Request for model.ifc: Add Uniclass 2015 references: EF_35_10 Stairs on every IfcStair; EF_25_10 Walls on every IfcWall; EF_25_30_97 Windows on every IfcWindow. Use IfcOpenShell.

First a look at what the model holds.

```python
import ifcopenshell

model = ifcopenshell.open("model.ifc")
print(model.schema)
print("classifications:", [c.Name for c in model.by_type("IfcClassification")])
for ifc_class in ("IfcDoor", "IfcRoof", "IfcStair", "IfcWall", "IfcWindow"):
    print(ifc_class, len(model.by_type(ifc_class)))
```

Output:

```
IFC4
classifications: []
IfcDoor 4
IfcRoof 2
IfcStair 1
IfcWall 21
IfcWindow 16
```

```python
import ifcopenshell
import ifcopenshell.api.classification

model = ifcopenshell.open("model.ifc")

system = ifcopenshell.api.classification.add_classification(model, classification="Uniclass 2015")

codes = {
    "IfcStair": ("EF_35_10", "Stairs"),
    "IfcWall": ("EF_25_10", "Walls"),
    "IfcWindow": ("EF_25_30_97", "Windows"),
}
for ifc_class, (code, name) in codes.items():
    products = model.by_type(ifc_class)
    ifcopenshell.api.classification.add_reference(
        model, products=products, classification=system, identification=code, name=name
    )
    print(code, len(products))

model.write("model_rev.ifc")
```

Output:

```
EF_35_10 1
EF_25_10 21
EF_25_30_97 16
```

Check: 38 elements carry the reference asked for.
